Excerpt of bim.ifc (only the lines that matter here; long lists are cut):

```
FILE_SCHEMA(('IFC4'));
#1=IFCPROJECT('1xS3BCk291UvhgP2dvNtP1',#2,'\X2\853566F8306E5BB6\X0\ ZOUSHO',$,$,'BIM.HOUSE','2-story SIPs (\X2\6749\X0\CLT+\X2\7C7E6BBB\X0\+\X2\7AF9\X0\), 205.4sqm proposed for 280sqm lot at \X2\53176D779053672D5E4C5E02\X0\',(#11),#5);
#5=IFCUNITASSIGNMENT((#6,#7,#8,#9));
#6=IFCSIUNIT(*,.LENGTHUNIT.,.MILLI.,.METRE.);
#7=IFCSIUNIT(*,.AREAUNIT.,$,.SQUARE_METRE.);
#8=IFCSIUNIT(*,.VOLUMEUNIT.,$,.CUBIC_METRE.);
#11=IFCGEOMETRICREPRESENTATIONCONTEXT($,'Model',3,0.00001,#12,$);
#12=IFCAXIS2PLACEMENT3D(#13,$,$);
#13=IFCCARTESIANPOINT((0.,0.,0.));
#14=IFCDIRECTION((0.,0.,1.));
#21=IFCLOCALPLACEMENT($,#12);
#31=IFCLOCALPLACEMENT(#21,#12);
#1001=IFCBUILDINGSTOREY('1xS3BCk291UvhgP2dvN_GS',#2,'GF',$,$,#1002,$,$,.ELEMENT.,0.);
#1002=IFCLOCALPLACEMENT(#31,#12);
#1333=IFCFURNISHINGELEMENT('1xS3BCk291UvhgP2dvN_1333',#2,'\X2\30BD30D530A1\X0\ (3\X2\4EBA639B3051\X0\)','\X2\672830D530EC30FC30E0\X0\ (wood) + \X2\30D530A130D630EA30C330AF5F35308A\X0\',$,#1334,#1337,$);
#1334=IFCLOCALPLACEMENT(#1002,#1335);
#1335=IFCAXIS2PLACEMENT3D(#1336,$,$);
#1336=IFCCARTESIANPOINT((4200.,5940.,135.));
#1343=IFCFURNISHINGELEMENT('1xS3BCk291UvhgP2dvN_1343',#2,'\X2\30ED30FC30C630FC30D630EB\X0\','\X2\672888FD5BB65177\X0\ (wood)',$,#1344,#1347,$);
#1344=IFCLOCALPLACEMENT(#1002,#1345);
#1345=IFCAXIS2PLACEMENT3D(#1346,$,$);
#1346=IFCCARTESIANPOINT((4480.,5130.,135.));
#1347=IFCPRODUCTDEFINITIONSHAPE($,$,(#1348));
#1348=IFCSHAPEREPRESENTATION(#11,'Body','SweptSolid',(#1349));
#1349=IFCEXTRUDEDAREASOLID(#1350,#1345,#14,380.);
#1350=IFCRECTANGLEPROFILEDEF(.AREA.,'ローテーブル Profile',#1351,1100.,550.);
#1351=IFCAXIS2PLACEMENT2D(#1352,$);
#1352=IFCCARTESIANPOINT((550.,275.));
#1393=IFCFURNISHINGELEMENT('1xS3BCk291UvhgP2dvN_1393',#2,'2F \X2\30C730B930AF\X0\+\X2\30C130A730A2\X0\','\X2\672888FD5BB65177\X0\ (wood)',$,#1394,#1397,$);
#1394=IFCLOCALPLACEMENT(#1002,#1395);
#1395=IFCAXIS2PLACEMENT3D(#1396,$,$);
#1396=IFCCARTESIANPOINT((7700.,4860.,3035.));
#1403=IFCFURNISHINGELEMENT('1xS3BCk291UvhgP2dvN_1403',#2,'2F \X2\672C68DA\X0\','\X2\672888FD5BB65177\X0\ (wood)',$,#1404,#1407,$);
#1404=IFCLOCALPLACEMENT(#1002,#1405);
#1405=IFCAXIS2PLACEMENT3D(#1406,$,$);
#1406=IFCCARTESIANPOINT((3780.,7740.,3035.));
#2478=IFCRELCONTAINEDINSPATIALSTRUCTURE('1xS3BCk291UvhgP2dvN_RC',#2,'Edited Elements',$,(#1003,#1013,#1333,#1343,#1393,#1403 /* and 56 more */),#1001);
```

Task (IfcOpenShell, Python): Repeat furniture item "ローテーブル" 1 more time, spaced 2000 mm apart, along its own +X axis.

```python
import ifcopenshell
import ifcopenshell.api.geometry
import ifcopenshell.api.root
import ifcopenshell.util.element
import ifcopenshell.util.placement
import ifcopenshell.util.unit

model = ifcopenshell.open("bim.ifc")
unit_scale = ifcopenshell.util.unit.calculate_unit_scale(model)


def reuse_history(source, copy):
    """copy_class also copies each property set's owner history, people and application; keep the originals."""
    for rel in copy.IsDefinedBy:
        if rel.is_a("IfcRelDefinesByProperties") and (history := rel.RelatingPropertyDefinition.OwnerHistory):
            rel.RelatingPropertyDefinition.OwnerHistory = source.OwnerHistory
            ifcopenshell.util.element.remove_deep2(model, history)


source = model.by_guid("1xS3BCk291UvhgP2dvN_1343")
base = ifcopenshell.util.placement.get_local_placement(source.ObjectPlacement)
step = base[:3, 0] * 2 / unit_scale

for i in range(1, 2):
    copy = ifcopenshell.api.root.copy_class(model, product=source)
    copy.Representation = ifcopenshell.util.element.copy_deep(
        model, source.Representation, exclude=["IfcGeometricRepresentationContext", "IfcRepresentationMap"]
    )
    reuse_history(source, copy)
    matrix = base.copy()
    matrix[:3, 3] += i * step
    print("added at", matrix[:3, 3].round(3) + 0.0)
    ifcopenshell.api.geometry.edit_object_placement(model, product=copy, matrix=matrix, is_si=False)

model.write("bim-out.ifc")
```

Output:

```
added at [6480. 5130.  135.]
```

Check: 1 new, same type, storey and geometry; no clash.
